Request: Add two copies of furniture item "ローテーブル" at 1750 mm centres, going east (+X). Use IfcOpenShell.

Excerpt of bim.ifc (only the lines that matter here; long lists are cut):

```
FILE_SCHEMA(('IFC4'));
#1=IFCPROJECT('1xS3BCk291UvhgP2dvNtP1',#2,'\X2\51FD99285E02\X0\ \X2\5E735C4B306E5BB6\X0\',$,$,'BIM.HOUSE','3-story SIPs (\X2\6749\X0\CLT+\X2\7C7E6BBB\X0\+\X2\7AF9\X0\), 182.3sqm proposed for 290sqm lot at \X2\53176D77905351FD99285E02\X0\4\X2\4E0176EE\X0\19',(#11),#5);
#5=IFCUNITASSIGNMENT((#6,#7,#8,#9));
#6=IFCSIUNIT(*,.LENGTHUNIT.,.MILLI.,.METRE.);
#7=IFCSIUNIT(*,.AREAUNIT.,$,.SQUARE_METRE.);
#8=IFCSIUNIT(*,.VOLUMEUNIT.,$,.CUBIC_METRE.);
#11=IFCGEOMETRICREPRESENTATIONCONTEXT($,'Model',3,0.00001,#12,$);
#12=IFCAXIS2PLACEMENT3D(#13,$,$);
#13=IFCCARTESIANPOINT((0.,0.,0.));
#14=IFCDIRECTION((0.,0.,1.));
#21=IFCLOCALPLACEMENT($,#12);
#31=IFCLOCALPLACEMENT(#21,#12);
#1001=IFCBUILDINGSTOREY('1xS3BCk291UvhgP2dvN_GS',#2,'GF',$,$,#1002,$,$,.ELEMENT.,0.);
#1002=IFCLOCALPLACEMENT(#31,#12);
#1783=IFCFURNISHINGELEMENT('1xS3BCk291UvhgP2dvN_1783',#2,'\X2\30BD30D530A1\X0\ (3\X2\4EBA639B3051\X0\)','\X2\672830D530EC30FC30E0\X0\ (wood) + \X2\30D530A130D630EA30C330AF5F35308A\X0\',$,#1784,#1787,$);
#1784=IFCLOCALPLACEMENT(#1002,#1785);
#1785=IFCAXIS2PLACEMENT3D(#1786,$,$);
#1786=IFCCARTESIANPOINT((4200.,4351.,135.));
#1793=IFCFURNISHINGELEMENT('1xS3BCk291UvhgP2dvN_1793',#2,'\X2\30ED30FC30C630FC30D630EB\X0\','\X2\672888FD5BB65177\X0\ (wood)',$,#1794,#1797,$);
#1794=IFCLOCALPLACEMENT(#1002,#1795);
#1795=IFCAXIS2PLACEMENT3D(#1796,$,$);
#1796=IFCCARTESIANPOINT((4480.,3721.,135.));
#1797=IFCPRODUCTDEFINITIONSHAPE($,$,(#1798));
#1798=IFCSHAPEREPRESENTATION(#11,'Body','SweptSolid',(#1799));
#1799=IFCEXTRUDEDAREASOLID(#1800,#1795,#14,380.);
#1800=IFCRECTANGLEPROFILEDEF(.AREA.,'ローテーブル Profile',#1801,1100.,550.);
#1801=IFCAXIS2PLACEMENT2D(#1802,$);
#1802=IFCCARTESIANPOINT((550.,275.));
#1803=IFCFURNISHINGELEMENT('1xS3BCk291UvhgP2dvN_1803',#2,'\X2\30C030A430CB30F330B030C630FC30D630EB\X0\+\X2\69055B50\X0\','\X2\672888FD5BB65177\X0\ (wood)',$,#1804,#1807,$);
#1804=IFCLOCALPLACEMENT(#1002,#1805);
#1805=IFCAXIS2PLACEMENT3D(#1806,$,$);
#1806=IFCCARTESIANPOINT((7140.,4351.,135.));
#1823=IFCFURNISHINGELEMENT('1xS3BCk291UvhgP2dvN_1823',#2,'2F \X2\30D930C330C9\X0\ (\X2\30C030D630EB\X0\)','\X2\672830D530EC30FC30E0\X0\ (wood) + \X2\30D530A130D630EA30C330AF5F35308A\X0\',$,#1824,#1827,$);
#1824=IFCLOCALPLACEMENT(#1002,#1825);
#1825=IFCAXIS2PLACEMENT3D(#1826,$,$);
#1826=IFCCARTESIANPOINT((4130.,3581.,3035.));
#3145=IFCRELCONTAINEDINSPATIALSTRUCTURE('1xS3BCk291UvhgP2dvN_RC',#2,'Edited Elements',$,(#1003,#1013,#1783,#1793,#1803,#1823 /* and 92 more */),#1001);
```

```python
import numpy as np
import ifcopenshell
import ifcopenshell.api.geometry
import ifcopenshell.api.root
import ifcopenshell.util.element
import ifcopenshell.util.placement

model = ifcopenshell.open("bim.ifc")


def reuse_history(source, copy):
    """copy_class also copies each property set's owner history, people and application; keep the originals."""
    for rel in copy.IsDefinedBy:
        if rel.is_a("IfcRelDefinesByProperties") and (history := rel.RelatingPropertyDefinition.OwnerHistory):
            rel.RelatingPropertyDefinition.OwnerHistory = source.OwnerHistory
            ifcopenshell.util.element.remove_deep2(model, history)


source = model.by_guid("1xS3BCk291UvhgP2dvN_1793")
base = ifcopenshell.util.placement.get_local_placement(source.ObjectPlacement)
step = np.array([1.0, 0.0, 0.0]) * 1750.0

for i in range(1, 3):
    copy = ifcopenshell.api.root.copy_class(model, product=source)
    copy.Representation = ifcopenshell.util.element.copy_deep(
        model, source.Representation, exclude=["IfcGeometricRepresentationContext", "IfcRepresentationMap"]
    )
    reuse_history(source, copy)
    matrix = base.copy()
    matrix[:3, 3] += i * step
    print("added at", matrix[:3, 3].round(3) + 0.0)
    ifcopenshell.api.geometry.edit_object_placement(model, product=copy, matrix=matrix, is_si=False)

model.write("bim_edited.ifc")
```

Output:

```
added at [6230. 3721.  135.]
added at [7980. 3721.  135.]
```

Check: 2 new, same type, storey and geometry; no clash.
